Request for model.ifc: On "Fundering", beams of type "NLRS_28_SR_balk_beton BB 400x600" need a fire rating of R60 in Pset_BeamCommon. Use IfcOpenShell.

First a look at what the model holds.

```python
import ifcopenshell
import ifcopenshell.util.element

model = ifcopenshell.open("model.ifc")
print(model.schema)
storey = next(s for s in model.by_type("IfcBuildingStorey") if s.Name == "Fundering")
beams = [e for e in ifcopenshell.util.element.get_decomposition(storey) if e.is_a("IfcBeam")]
seen = {}
for e in beams:
    element_type = ifcopenshell.util.element.get_type(e)
    key = (element_type.Name if element_type != e and element_type else None, ifcopenshell.util.element.get_pset(e, "Pset_BeamCommon", "FireRating"))
    seen[key] = seen.get(key, 0) + 1
for (name, value), count in sorted(seen.items(), key=str):
    print(count, "x", name, "|", value)
```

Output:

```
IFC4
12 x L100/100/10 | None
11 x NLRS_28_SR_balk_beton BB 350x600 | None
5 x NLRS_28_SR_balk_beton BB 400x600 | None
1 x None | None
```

```python
import ifcopenshell
import ifcopenshell.api.pset
import ifcopenshell.util.element

model = ifcopenshell.open("model.ifc")

storey = next(s for s in model.by_type("IfcBuildingStorey") if s.Name == "Fundering")
beams = [e for e in ifcopenshell.util.element.get_decomposition(storey) if e.is_a("IfcBeam")]

count = 0
for e in beams:
    element_type = ifcopenshell.util.element.get_type(e)
    if element_type in (None, e) or element_type.Name != "NLRS_28_SR_balk_beton BB 400x600":
        continue
    # add_pset returns the element's existing set when there is one.
    pset = ifcopenshell.api.pset.add_pset(model, product=e, name="Pset_BeamCommon")
    ifcopenshell.api.pset.edit_pset(model, pset=pset, properties={"FireRating": "R60"})
    count += 1

print(count, "beams updated")

model.write("model_v2.ifc")
```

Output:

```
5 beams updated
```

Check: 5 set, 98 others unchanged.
